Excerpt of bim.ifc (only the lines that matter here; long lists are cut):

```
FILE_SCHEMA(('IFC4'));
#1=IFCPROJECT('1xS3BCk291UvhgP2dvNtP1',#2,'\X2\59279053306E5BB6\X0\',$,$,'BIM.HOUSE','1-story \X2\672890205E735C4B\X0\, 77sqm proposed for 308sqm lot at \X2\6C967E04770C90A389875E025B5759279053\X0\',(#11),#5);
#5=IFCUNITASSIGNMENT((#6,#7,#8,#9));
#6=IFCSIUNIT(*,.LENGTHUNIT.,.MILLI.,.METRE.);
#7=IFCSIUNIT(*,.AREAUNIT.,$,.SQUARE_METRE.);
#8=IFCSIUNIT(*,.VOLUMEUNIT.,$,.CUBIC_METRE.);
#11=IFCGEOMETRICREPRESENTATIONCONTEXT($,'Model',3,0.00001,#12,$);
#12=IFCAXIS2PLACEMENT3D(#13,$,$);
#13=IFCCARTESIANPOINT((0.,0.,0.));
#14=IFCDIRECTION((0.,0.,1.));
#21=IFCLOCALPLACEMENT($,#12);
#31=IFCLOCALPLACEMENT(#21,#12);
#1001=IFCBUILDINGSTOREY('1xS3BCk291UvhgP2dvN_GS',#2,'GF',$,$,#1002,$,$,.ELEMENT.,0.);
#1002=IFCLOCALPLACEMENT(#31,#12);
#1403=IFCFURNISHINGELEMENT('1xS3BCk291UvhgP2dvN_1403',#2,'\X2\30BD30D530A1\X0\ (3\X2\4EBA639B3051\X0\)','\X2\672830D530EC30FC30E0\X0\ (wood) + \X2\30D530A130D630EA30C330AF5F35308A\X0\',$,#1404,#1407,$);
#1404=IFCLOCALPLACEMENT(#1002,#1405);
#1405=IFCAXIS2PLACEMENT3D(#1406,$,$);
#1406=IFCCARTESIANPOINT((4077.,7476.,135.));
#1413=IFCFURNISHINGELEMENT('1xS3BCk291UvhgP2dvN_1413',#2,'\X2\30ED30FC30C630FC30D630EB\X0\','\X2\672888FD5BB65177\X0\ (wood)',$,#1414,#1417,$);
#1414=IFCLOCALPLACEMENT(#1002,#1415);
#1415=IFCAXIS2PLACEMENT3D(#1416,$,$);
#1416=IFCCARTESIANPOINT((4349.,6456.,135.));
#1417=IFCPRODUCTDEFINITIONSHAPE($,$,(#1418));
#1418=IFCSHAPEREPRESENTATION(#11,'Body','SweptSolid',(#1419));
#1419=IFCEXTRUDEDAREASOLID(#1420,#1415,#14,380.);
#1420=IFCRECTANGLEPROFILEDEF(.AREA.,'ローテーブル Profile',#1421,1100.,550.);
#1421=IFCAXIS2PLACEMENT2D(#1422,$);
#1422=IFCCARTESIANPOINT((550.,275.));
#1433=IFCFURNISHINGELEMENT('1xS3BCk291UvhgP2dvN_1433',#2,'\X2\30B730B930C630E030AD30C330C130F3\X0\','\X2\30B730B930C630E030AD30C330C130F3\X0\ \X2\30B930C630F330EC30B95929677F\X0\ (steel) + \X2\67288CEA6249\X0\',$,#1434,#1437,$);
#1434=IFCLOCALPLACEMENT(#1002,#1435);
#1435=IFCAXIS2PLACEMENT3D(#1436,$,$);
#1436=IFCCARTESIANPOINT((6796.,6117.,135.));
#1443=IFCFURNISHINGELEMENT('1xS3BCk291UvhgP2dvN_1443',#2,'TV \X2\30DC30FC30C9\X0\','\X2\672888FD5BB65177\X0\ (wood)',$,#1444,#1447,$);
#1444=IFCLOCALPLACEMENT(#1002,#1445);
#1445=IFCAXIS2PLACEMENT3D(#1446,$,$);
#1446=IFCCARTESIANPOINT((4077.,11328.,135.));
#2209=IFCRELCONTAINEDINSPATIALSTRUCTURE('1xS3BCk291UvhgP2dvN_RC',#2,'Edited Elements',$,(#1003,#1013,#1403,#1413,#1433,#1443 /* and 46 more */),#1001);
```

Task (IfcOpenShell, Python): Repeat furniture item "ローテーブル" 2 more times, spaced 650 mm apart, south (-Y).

```python
import numpy as np
import ifcopenshell
import ifcopenshell.api.geometry
import ifcopenshell.api.root
import ifcopenshell.util.element
import ifcopenshell.util.placement
import ifcopenshell.util.unit

model = ifcopenshell.open("bim.ifc")
unit_scale = ifcopenshell.util.unit.calculate_unit_scale(model)


def reuse_history(source, copy):
    """copy_class also copies each property set's owner history, people and application; keep the originals."""
    for rel in copy.IsDefinedBy:
        if rel.is_a("IfcRelDefinesByProperties") and (history := rel.RelatingPropertyDefinition.OwnerHistory):
            rel.RelatingPropertyDefinition.OwnerHistory = source.OwnerHistory
            ifcopenshell.util.element.remove_deep2(model, history)


source = model.by_id(1413)
base = ifcopenshell.util.placement.get_local_placement(source.ObjectPlacement)
step = np.array([0.0, -1.0, 0.0]) * 0.65 / unit_scale

for i in range(1, 3):
    copy = ifcopenshell.api.root.copy_class(model, product=source)
    copy.Representation = ifcopenshell.util.element.copy_deep(
        model, source.Representation, exclude=["IfcGeometricRepresentationContext", "IfcRepresentationMap"]
    )
    reuse_history(source, copy)
    matrix = base.copy()
    matrix[:3, 3] += i * step
    print("added at", matrix[:3, 3].round(3) + 0.0)
    ifcopenshell.api.geometry.edit_object_placement(model, product=copy, matrix=matrix, is_si=False)

model.write("bim_v2.ifc")
```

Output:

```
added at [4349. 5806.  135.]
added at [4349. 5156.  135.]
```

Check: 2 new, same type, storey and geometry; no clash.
